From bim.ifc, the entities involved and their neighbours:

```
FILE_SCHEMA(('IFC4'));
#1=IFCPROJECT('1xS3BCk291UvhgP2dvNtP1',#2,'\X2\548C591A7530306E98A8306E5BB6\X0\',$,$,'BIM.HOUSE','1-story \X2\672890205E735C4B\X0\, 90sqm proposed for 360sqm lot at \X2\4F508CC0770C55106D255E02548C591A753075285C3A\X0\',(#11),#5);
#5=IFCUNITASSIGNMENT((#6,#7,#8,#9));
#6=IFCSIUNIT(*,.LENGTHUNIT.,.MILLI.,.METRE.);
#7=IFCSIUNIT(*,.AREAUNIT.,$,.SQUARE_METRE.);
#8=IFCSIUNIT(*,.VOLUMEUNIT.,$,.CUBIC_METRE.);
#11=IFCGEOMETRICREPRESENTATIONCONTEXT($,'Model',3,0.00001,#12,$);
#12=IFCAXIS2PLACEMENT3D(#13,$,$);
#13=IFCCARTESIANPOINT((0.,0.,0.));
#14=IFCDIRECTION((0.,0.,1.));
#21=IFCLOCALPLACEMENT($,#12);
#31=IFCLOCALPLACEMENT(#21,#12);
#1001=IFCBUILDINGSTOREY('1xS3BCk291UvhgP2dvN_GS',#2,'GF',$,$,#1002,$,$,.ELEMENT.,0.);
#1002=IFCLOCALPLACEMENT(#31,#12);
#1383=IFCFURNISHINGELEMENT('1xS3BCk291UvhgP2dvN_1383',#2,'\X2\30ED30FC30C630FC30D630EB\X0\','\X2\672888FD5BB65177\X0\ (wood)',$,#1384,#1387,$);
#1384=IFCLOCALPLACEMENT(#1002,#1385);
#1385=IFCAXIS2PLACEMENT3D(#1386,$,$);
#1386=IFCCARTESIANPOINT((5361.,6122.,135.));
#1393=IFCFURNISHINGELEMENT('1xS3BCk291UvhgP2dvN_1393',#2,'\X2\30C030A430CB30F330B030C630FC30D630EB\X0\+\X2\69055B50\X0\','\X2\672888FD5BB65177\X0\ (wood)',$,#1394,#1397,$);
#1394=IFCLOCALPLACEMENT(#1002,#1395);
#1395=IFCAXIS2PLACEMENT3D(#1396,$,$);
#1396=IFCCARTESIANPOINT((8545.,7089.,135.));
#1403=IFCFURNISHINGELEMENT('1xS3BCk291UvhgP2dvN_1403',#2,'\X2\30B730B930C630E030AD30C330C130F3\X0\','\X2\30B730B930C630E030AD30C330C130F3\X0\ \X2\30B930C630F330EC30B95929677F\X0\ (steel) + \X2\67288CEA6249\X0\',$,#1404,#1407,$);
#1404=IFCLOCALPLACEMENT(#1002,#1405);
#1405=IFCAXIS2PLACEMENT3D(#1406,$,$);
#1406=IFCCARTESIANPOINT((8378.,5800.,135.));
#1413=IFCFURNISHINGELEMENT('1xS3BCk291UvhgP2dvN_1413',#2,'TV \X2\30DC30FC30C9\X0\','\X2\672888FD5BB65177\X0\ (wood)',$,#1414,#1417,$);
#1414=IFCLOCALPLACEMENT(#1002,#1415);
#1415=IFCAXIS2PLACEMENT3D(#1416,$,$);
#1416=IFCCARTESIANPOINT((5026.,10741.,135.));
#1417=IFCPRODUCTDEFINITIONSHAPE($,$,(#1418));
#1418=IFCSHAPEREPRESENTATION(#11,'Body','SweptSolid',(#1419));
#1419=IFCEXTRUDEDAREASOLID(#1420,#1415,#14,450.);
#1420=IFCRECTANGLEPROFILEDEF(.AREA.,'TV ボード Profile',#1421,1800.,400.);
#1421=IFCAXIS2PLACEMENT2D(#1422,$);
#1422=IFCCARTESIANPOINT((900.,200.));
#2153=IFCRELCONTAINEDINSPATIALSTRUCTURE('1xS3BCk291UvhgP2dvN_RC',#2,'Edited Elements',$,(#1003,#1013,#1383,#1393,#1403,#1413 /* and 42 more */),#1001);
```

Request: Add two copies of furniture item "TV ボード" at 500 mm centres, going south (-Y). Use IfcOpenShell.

```python
import numpy as np
import ifcopenshell
import ifcopenshell.api.geometry
import ifcopenshell.api.root
import ifcopenshell.util.element
import ifcopenshell.util.placement
import ifcopenshell.util.unit

model = ifcopenshell.open("bim.ifc")
unit_scale = ifcopenshell.util.unit.calculate_unit_scale(model)


def reuse_history(source, copy):
    """copy_class also copies each property set's owner history, people and application; keep the originals."""
    for rel in copy.IsDefinedBy:
        if rel.is_a("IfcRelDefinesByProperties") and (history := rel.RelatingPropertyDefinition.OwnerHistory):
            rel.RelatingPropertyDefinition.OwnerHistory = source.OwnerHistory
            ifcopenshell.util.element.remove_deep2(model, history)


source = model.by_guid("1xS3BCk291UvhgP2dvN_1413")
base = ifcopenshell.util.placement.get_local_placement(source.ObjectPlacement)
step = np.array([0.0, -1.0, 0.0]) * 0.5 / unit_scale

for i in range(1, 3):
    copy = ifcopenshell.api.root.copy_class(model, product=source)
    copy.Representation = ifcopenshell.util.element.copy_deep(
        model, source.Representation, exclude=["IfcGeometricRepresentationContext", "IfcRepresentationMap"]
    )
    reuse_history(source, copy)
    matrix = base.copy()
    matrix[:3, 3] += i * step
    print("added at", matrix[:3, 3].round(3) + 0.0)
    ifcopenshell.api.geometry.edit_object_placement(model, product=copy, matrix=matrix, is_si=False)

model.write("bim-out.ifc")
```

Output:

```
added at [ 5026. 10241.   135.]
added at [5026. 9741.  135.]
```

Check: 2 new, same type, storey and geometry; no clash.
